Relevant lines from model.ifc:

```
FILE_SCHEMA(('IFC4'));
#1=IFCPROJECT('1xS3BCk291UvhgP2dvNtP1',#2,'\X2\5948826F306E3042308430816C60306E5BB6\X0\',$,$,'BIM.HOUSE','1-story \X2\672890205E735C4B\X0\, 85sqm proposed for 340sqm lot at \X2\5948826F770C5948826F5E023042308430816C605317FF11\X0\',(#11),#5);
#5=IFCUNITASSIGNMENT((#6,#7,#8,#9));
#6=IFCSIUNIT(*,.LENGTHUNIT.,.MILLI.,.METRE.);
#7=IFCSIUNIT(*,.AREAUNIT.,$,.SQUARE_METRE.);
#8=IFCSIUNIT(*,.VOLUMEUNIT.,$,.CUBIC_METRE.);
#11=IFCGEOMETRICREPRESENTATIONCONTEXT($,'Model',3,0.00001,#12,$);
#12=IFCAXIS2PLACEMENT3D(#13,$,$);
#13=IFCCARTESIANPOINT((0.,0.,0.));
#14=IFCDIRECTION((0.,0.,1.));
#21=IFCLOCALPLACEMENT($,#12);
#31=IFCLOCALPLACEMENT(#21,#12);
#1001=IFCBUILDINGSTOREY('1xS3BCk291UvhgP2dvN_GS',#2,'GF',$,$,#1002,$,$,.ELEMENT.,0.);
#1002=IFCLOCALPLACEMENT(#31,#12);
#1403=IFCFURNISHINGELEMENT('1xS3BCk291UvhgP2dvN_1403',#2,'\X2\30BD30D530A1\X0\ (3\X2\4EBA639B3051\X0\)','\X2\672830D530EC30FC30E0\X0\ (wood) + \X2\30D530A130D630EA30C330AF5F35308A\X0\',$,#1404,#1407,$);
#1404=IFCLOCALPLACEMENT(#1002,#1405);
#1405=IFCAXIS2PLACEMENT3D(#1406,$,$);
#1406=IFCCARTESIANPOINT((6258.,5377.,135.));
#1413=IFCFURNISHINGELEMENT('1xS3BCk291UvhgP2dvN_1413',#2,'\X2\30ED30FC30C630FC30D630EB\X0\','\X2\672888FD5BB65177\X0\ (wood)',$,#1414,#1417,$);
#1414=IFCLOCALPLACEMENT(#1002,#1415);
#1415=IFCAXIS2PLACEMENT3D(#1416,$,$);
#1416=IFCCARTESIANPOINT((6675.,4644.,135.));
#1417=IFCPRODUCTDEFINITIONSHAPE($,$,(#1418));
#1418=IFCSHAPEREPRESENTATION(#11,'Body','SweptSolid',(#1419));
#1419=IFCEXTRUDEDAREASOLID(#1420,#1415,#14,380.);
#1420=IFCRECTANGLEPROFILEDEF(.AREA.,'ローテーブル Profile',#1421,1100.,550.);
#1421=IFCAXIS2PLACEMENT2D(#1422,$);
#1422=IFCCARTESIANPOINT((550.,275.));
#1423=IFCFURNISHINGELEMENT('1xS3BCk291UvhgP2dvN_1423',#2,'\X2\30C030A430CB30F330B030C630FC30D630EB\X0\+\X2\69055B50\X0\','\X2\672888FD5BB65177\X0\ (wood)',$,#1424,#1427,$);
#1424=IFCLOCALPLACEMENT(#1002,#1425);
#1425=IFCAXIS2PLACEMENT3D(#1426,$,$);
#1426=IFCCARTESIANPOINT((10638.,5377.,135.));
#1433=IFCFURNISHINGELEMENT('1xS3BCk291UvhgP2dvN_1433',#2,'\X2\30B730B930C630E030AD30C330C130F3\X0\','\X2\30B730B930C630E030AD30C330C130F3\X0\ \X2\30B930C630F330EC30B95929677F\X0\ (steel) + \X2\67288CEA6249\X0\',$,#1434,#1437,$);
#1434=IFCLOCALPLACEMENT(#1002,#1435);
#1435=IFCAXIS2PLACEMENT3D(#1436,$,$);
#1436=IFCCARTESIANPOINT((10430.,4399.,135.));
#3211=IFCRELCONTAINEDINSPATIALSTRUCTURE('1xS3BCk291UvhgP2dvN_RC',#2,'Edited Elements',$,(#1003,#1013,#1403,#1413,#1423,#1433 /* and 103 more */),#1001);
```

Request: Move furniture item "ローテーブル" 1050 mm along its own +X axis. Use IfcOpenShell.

```python
import ifcopenshell
import ifcopenshell.api.geometry
import ifcopenshell.util.placement
import ifcopenshell.util.unit

model = ifcopenshell.open("model.ifc")
unit_scale = ifcopenshell.util.unit.calculate_unit_scale(model)

item = model.by_guid("1xS3BCk291UvhgP2dvN_1413")
matrix = ifcopenshell.util.placement.get_local_placement(item.ObjectPlacement)
matrix[:3, 3] += matrix[:3, 0] * 1.05 / unit_scale
ifcopenshell.api.geometry.edit_object_placement(model, product=item, matrix=matrix, is_si=False)

print(ifcopenshell.util.placement.get_local_placement(item.ObjectPlacement).round(3) + 0.0)

model.write("model-out.ifc")
```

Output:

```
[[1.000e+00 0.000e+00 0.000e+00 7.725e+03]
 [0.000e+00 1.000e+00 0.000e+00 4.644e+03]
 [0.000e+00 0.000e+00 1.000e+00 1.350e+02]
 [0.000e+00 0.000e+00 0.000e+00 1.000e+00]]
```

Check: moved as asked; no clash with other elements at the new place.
